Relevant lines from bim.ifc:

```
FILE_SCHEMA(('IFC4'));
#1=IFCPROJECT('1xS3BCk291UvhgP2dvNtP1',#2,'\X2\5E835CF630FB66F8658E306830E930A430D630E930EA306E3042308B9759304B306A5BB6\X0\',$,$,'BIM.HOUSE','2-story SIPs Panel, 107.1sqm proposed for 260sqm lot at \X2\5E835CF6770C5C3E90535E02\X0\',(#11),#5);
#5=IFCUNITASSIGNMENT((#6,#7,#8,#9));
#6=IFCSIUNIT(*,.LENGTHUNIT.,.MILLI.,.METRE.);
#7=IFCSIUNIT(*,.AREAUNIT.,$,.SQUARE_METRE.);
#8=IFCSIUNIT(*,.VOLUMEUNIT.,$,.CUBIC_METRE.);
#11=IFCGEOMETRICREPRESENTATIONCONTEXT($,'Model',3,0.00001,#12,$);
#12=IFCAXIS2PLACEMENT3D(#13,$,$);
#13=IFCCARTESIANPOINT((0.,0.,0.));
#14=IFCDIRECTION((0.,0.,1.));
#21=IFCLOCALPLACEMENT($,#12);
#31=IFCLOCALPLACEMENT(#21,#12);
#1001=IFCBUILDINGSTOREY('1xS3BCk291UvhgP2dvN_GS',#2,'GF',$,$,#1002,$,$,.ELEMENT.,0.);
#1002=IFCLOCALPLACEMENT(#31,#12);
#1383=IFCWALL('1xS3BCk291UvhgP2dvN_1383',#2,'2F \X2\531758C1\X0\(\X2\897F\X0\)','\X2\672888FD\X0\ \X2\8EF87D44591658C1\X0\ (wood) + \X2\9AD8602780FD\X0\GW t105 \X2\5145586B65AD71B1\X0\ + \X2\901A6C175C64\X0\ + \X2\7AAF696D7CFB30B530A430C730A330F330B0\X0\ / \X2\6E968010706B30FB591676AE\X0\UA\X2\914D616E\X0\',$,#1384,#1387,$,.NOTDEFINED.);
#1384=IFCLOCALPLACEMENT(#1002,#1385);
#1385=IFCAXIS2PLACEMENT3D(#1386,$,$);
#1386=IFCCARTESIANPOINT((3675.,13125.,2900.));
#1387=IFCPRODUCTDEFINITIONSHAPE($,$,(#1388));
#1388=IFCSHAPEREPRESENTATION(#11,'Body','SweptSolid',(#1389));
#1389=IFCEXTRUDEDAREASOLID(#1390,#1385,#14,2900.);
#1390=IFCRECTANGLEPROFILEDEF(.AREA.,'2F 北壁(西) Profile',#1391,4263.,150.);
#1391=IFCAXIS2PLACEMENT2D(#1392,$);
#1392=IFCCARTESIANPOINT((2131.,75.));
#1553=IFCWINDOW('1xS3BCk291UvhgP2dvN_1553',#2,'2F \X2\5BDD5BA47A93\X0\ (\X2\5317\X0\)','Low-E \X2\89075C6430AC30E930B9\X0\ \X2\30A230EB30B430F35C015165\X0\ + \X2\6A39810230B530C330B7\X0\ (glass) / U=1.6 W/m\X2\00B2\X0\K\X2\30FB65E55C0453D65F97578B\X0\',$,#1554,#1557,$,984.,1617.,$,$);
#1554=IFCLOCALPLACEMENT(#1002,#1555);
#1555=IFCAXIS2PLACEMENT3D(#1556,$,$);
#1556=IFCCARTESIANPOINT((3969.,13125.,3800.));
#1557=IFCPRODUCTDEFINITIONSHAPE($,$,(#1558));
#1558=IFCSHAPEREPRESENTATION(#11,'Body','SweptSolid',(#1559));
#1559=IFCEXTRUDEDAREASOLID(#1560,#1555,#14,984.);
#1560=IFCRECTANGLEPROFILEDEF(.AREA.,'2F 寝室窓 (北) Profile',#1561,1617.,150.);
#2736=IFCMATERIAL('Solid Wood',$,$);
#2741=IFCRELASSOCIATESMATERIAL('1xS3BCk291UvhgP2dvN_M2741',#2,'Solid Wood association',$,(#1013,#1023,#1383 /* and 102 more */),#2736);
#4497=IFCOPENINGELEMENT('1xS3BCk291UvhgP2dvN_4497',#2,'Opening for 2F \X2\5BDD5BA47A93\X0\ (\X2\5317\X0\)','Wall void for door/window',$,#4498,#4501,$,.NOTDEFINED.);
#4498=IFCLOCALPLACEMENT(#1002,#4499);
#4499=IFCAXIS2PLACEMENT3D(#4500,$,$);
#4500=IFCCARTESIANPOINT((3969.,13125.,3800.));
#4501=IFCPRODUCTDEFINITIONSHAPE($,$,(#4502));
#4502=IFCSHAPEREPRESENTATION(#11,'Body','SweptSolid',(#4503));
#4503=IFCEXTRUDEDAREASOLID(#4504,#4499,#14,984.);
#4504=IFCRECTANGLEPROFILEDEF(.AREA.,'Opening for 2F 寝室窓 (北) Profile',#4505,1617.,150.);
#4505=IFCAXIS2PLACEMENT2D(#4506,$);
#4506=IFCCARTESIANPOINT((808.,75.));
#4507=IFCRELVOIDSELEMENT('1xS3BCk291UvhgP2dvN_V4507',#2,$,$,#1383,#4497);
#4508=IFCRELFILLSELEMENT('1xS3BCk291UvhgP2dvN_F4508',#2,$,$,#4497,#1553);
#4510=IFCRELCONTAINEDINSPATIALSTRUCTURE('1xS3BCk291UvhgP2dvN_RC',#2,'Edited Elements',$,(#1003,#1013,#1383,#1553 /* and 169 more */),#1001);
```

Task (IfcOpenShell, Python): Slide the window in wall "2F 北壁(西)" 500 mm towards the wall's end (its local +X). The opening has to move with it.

```python
import ifcopenshell
import ifcopenshell.api.geometry
import ifcopenshell.util.placement

model = ifcopenshell.open("bim.ifc")

window = model.by_guid("1xS3BCk291UvhgP2dvN_1553")
opening = window.FillsVoids[0].RelatingOpeningElement
wall = opening.VoidsElements[0].RelatingBuildingElement

wall_matrix = ifcopenshell.util.placement.get_local_placement(wall.ObjectPlacement)
shift = wall_matrix[:3, 0] * 500.0
before = ifcopenshell.util.placement.get_local_placement(window.ObjectPlacement)[:3, 3].copy()

# The window is not placed relative to its opening, so move both.
for product in (opening, window):
    matrix = ifcopenshell.util.placement.get_local_placement(product.ObjectPlacement)
    matrix[:3, 3] += shift
    ifcopenshell.api.geometry.edit_object_placement(model, product=product, matrix=matrix, is_si=False)

after = ifcopenshell.util.placement.get_local_placement(window.ObjectPlacement)[:3, 3]
print("window moved by", (after - before).round(3) + 0.0)

model.write("bim_updated.ifc")
```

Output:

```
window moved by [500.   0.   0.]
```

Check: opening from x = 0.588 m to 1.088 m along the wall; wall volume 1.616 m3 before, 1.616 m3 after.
